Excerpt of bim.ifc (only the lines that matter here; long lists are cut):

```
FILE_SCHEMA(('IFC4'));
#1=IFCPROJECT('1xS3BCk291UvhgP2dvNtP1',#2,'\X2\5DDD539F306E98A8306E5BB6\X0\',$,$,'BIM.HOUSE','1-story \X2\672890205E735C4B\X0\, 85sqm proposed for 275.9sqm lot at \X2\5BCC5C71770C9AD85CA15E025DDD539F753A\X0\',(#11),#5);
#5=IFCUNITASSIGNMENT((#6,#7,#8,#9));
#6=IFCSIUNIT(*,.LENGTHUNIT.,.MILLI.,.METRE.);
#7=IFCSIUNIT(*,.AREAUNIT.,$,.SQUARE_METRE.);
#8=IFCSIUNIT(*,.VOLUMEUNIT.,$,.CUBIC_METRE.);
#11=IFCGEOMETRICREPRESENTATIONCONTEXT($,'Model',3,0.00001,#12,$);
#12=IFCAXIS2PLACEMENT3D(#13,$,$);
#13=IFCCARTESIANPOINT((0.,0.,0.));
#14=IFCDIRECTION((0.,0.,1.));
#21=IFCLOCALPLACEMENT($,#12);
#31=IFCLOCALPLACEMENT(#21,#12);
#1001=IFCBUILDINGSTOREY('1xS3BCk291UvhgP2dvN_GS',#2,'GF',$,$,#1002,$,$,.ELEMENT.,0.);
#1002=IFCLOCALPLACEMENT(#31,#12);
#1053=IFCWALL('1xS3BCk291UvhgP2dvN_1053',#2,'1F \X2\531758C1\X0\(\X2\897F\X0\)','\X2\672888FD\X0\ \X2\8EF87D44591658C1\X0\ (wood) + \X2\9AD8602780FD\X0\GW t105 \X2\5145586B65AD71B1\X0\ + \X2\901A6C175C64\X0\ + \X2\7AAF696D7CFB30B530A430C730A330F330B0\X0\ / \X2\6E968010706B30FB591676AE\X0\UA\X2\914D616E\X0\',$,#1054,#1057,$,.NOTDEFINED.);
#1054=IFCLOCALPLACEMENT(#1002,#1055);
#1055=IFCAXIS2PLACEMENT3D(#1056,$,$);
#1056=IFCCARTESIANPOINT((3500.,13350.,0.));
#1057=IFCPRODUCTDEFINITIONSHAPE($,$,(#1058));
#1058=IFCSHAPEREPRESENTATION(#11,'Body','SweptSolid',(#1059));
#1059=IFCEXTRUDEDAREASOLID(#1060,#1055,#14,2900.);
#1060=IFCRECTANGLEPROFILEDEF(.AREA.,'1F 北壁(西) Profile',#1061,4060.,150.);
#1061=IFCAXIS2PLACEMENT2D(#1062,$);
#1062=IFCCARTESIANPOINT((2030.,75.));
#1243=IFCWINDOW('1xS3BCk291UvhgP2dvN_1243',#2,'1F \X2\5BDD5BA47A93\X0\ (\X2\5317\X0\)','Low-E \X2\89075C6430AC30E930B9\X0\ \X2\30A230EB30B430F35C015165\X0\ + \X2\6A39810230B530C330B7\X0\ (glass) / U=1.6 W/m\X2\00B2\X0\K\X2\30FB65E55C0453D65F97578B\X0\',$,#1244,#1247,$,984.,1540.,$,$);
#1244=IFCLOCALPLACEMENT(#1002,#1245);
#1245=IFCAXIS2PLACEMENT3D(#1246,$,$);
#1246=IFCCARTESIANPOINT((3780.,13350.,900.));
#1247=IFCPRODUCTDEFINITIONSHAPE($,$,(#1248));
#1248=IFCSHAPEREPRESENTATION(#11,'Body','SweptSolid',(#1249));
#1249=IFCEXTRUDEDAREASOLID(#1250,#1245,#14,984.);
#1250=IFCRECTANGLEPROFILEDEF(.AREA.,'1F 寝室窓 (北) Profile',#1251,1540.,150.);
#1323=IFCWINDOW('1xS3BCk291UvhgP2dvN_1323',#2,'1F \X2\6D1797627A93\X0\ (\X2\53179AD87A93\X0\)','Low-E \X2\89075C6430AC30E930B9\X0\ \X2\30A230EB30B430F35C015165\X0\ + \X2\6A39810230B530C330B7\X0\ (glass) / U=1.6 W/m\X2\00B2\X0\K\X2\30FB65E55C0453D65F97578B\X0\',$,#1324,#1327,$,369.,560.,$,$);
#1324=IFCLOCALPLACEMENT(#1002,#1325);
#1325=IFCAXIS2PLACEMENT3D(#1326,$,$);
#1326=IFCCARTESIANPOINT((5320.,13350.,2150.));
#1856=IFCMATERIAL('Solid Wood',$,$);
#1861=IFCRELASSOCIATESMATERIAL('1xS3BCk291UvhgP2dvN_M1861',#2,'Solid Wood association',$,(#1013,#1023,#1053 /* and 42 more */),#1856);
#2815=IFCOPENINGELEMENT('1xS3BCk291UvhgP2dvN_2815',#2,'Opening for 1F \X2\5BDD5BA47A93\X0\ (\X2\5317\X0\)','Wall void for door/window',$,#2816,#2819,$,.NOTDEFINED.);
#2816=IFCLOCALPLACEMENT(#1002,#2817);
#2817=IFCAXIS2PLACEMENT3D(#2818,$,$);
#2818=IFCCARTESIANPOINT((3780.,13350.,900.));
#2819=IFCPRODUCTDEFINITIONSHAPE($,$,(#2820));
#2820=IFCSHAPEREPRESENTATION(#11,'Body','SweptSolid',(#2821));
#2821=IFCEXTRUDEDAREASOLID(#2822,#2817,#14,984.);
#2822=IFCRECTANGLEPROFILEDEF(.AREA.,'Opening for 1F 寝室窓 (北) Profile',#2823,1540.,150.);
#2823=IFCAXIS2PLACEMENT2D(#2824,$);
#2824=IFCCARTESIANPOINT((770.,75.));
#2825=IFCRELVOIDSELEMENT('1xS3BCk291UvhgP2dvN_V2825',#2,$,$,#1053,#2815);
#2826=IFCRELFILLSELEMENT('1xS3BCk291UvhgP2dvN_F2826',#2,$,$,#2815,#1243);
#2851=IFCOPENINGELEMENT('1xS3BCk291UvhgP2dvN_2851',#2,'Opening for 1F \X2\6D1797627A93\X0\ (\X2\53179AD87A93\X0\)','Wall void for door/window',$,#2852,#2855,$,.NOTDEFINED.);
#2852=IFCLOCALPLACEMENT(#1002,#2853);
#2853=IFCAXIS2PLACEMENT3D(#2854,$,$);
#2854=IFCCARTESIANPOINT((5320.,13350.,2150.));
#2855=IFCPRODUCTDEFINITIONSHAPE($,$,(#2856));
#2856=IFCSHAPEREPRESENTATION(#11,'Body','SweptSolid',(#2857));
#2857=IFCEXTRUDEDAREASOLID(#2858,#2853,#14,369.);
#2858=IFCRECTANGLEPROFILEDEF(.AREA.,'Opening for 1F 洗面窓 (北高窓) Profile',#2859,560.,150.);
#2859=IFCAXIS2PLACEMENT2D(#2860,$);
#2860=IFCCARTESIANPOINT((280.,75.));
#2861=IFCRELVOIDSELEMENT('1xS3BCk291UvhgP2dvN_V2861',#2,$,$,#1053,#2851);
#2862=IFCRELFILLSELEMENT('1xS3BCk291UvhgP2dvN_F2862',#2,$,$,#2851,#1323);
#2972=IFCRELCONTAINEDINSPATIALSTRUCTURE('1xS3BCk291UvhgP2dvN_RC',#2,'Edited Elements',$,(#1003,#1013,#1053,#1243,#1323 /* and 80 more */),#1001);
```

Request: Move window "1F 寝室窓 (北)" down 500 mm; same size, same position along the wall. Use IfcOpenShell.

```python
import numpy as np
import ifcopenshell
import ifcopenshell.api.geometry
import ifcopenshell.util.placement
import ifcopenshell.util.unit

model = ifcopenshell.open("bim.ifc")
unit_scale = ifcopenshell.util.unit.calculate_unit_scale(model)

window = model.by_id(1243)
opening = window.FillsVoids[0].RelatingOpeningElement
dz = -0.5 / unit_scale

shift = np.array([0.0, 0.0, dz])
# The window is not placed relative to its opening, so move both.
for product in (opening, window):
    matrix = ifcopenshell.util.placement.get_local_placement(product.ObjectPlacement)
    matrix[:3, 3] += shift
    ifcopenshell.api.geometry.edit_object_placement(model, product=product, matrix=matrix, is_si=False)

print(f"moved by {dz * unit_scale:+.3f} m")

model.write("bim_v2.ifc")
```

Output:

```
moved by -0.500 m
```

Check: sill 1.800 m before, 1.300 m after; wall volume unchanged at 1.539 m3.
